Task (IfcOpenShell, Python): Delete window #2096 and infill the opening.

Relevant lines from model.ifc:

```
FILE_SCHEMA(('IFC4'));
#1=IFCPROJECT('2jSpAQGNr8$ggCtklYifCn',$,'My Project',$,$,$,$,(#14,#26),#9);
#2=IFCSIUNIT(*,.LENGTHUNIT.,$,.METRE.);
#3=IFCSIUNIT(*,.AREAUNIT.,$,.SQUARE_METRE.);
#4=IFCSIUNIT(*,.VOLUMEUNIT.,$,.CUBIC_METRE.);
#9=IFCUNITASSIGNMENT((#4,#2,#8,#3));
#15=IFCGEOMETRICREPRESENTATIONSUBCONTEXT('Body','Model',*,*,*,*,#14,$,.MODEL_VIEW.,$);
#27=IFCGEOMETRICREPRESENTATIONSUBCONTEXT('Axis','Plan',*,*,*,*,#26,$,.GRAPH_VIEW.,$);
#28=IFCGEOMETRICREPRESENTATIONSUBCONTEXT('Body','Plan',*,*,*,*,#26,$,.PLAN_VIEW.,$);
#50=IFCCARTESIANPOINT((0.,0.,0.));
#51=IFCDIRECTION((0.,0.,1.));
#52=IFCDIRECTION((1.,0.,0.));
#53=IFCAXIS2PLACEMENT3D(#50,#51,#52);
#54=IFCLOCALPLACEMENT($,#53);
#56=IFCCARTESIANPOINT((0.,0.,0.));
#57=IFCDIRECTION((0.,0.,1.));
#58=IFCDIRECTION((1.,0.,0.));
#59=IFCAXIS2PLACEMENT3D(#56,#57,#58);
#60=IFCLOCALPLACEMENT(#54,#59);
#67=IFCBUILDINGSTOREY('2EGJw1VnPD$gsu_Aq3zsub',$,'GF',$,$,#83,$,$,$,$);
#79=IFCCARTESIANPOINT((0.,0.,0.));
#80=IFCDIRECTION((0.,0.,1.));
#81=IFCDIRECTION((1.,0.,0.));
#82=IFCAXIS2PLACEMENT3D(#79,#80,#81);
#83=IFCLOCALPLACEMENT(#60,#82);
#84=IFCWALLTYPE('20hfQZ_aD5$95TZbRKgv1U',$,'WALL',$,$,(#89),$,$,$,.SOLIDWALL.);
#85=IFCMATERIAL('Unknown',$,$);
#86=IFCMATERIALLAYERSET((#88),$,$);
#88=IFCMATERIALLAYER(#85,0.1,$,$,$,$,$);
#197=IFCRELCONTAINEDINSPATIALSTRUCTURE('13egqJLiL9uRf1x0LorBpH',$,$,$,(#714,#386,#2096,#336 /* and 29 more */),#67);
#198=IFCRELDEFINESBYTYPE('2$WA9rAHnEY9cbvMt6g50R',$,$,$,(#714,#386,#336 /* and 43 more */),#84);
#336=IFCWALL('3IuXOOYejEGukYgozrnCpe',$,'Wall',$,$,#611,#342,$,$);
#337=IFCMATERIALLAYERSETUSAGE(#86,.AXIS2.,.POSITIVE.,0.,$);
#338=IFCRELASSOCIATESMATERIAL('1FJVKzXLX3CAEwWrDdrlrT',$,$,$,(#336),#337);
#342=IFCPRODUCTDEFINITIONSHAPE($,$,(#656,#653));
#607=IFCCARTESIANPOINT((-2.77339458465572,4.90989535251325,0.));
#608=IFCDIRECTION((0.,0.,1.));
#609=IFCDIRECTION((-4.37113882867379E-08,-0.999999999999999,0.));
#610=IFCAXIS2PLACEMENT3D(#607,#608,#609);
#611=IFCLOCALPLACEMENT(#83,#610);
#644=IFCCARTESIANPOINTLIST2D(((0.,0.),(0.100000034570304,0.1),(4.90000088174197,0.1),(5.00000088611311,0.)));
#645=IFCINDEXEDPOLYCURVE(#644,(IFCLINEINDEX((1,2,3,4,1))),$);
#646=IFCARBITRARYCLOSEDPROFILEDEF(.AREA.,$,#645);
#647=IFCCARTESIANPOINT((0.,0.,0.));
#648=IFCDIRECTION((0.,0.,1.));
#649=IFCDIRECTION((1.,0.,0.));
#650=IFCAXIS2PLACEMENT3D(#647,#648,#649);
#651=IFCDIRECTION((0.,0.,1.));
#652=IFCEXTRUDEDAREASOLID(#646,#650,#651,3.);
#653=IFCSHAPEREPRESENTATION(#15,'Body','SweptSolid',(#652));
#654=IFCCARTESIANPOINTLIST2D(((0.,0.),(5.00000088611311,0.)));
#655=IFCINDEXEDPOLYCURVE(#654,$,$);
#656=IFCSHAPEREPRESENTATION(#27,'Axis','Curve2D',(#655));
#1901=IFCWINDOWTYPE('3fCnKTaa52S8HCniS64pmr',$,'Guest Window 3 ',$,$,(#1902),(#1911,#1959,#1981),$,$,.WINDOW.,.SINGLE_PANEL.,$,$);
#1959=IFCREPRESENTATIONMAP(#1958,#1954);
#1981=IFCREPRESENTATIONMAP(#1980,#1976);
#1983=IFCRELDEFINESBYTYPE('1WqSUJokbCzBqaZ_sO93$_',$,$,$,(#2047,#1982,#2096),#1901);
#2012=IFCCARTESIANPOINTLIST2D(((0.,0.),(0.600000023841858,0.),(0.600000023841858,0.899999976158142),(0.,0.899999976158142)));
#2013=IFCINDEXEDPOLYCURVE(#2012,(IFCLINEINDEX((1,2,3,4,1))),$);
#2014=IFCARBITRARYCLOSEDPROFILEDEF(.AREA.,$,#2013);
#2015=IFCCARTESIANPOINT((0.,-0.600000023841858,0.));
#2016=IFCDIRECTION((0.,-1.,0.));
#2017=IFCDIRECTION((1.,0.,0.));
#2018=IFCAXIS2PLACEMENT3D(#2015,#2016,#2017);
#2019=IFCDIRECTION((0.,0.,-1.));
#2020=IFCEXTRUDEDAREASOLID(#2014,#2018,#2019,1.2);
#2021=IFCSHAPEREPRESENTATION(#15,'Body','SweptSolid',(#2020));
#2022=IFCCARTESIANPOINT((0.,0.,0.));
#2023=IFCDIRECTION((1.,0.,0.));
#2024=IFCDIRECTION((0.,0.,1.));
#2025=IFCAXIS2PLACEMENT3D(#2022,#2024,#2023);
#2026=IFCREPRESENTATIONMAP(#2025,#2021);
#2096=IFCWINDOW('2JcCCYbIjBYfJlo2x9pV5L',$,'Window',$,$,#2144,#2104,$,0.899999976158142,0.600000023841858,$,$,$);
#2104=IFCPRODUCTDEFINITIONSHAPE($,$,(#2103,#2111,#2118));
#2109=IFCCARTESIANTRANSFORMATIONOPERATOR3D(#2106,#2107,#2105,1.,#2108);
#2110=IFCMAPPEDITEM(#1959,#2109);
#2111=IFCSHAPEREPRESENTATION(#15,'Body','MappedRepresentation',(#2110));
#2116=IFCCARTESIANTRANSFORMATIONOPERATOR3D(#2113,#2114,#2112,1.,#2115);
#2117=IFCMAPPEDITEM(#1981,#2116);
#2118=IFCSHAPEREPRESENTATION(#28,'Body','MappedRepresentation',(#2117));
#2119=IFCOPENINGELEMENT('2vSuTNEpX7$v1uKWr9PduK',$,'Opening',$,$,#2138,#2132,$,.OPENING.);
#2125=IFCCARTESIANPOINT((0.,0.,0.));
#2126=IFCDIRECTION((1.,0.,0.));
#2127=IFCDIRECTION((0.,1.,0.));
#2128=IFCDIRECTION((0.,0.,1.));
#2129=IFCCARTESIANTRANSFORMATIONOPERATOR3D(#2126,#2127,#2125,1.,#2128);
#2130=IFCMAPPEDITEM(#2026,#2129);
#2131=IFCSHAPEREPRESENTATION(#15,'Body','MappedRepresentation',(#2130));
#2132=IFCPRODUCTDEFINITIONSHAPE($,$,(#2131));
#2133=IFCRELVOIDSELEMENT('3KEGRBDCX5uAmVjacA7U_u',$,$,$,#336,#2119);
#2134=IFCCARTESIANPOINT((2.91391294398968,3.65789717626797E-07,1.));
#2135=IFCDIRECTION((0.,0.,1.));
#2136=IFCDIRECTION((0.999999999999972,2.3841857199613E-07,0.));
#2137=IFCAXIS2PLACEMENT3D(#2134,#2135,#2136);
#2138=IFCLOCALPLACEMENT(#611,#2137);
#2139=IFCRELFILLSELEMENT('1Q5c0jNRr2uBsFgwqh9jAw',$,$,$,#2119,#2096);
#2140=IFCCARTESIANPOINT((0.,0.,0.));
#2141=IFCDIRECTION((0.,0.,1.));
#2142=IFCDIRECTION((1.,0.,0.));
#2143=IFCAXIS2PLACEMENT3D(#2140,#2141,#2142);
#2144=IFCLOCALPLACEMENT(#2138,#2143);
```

```python
import ifcopenshell
import ifcopenshell.api.feature
import ifcopenshell.api.root
import ifcopenshell.geom
import ifcopenshell.util.shape

model = ifcopenshell.open("model.ifc")
settings = ifcopenshell.geom.settings()


def volume(element):
    """Net volume in cubic metres, openings subtracted."""
    shape = ifcopenshell.geom.create_shape(settings, element)
    return ifcopenshell.util.shape.get_volume(shape.geometry)


window = model.by_id(2096)
opening = window.FillsVoids[0].RelatingOpeningElement
wall = opening.VoidsElements[0].RelatingBuildingElement
before = volume(wall)

ifcopenshell.api.root.remove_product(model, product=window)
ifcopenshell.api.feature.remove_feature(model, feature=opening)

after = volume(wall)

print(f"wall volume {before:.3f} -> {after:.3f} m3")

model.write("model-out.ifc")
```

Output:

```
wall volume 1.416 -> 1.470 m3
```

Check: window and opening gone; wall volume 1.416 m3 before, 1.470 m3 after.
